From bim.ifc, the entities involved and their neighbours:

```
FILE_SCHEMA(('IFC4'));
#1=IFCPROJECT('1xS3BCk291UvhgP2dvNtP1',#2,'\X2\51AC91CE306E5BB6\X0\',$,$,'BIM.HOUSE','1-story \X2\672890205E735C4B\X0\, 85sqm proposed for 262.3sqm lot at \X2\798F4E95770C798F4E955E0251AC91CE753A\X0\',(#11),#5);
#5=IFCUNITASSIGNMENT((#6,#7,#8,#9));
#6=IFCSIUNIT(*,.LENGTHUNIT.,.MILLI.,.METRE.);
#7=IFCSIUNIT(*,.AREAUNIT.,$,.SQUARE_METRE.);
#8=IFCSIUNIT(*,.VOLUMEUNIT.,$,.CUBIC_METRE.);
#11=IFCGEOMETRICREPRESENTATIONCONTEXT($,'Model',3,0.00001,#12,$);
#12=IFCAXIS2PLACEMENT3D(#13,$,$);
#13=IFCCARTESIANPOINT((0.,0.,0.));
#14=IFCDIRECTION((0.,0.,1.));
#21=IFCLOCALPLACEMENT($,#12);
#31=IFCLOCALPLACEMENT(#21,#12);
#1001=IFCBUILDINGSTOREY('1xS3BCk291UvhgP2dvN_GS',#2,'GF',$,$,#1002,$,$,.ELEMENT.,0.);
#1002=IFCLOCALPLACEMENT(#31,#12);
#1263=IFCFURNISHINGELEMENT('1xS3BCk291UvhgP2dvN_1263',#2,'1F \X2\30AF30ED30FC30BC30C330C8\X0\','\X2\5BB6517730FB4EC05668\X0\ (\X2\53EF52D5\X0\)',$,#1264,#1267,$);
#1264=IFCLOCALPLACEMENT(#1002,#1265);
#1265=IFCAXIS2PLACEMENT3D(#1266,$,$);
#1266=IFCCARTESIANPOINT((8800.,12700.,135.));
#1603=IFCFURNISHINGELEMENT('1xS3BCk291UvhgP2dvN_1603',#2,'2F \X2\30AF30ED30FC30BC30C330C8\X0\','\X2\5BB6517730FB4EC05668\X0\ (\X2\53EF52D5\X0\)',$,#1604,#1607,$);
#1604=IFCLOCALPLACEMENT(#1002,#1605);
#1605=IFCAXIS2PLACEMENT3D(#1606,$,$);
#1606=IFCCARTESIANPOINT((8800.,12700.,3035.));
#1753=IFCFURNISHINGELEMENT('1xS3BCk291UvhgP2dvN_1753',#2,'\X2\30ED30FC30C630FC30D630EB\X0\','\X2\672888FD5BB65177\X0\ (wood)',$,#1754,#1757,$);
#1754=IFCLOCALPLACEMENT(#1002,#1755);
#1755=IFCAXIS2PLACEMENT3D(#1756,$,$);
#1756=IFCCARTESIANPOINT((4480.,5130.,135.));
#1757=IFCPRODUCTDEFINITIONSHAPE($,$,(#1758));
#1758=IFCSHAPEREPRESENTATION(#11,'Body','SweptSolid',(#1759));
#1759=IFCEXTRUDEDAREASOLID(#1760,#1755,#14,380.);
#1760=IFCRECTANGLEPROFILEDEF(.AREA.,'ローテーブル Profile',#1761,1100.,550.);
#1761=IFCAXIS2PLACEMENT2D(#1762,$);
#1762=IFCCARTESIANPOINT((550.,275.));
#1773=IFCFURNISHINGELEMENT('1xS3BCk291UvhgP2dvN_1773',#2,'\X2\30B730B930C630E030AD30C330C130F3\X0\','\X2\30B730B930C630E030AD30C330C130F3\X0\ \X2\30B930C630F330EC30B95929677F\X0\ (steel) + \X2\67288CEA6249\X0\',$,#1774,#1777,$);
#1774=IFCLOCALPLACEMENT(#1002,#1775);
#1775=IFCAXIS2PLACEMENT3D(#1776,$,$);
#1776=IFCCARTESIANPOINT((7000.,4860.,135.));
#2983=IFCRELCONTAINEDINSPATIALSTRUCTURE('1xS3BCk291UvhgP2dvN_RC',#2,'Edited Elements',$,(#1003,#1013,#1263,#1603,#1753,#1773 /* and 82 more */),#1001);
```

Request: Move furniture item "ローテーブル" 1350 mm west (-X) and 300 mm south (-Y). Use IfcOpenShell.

```python
import ifcopenshell
import ifcopenshell.api.geometry
import ifcopenshell.util.placement

model = ifcopenshell.open("bim.ifc")

item = model.by_guid("1xS3BCk291UvhgP2dvN_1753")
matrix = ifcopenshell.util.placement.get_local_placement(item.ObjectPlacement)
matrix[0, 3] -= 1350.0
matrix[1, 3] -= 300.0
ifcopenshell.api.geometry.edit_object_placement(model, product=item, matrix=matrix, is_si=False)

print(ifcopenshell.util.placement.get_local_placement(item.ObjectPlacement).round(3) + 0.0)

model.write("bim_v2.ifc")
```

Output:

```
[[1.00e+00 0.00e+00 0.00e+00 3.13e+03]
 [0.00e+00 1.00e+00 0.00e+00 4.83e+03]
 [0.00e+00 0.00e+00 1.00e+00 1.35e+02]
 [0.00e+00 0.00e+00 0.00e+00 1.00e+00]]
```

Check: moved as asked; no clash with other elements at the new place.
